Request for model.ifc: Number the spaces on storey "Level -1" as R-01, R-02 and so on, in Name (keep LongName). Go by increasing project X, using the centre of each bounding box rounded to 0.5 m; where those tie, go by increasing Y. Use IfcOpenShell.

First a look at what the model holds.

```python
import ifcopenshell
import ifcopenshell.util.element
import ifcopenshell.util.placement

model = ifcopenshell.open("model.ifc")
print(model.schema)
storey = next(s for s in model.by_type("IfcBuildingStorey") if s.Name == "Level -1")
spaces = [e for e in ifcopenshell.util.element.get_decomposition(storey) if e.is_a("IfcSpace")]
for e in sorted(spaces, key=lambda e: e.id()):
    origin = ifcopenshell.util.placement.get_local_placement(e.ObjectPlacement)[:3, 3]
    print(e.id(), e.Name, e.LongName, origin.round(2) + 0.0, sep=" | ")
```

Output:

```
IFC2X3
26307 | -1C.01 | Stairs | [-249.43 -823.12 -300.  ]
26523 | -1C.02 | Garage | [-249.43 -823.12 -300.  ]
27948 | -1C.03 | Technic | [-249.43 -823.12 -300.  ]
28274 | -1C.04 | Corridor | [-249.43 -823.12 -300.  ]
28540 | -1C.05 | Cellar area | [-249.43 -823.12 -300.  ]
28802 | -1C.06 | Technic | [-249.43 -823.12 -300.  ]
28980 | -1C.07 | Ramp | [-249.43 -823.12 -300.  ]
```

```python
import ifcopenshell
import ifcopenshell.geom
import ifcopenshell.util.element
import ifcopenshell.util.shape

model = ifcopenshell.open("model.ifc")
settings = ifcopenshell.geom.settings()
settings.set("use-world-coords", True)


def centre(element):
    shape = ifcopenshell.geom.create_shape(settings, element)
    return ifcopenshell.util.shape.get_bbox_centroid(shape.geometry)


storey = next(s for s in model.by_type("IfcBuildingStorey") if s.Name == "Level -1")
spaces = [e for e in ifcopenshell.util.element.get_decomposition(storey) if e.is_a("IfcSpace")]

# Insertion points can sit at a corner or the storey origin, so sort by the geometry (in metres).
centres = {e: centre(e) for e in spaces}
spaces.sort(key=lambda e: (round(centres[e][0] / 0.5), centres[e][1]))

for i, e in enumerate(spaces, start=1):
    number = f"R-{i:02d}"
    e.Name = number
    print(e.id(), number)

model.write("model_rev.ifc")
```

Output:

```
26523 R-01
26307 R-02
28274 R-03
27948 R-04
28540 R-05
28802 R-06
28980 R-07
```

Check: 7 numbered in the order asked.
